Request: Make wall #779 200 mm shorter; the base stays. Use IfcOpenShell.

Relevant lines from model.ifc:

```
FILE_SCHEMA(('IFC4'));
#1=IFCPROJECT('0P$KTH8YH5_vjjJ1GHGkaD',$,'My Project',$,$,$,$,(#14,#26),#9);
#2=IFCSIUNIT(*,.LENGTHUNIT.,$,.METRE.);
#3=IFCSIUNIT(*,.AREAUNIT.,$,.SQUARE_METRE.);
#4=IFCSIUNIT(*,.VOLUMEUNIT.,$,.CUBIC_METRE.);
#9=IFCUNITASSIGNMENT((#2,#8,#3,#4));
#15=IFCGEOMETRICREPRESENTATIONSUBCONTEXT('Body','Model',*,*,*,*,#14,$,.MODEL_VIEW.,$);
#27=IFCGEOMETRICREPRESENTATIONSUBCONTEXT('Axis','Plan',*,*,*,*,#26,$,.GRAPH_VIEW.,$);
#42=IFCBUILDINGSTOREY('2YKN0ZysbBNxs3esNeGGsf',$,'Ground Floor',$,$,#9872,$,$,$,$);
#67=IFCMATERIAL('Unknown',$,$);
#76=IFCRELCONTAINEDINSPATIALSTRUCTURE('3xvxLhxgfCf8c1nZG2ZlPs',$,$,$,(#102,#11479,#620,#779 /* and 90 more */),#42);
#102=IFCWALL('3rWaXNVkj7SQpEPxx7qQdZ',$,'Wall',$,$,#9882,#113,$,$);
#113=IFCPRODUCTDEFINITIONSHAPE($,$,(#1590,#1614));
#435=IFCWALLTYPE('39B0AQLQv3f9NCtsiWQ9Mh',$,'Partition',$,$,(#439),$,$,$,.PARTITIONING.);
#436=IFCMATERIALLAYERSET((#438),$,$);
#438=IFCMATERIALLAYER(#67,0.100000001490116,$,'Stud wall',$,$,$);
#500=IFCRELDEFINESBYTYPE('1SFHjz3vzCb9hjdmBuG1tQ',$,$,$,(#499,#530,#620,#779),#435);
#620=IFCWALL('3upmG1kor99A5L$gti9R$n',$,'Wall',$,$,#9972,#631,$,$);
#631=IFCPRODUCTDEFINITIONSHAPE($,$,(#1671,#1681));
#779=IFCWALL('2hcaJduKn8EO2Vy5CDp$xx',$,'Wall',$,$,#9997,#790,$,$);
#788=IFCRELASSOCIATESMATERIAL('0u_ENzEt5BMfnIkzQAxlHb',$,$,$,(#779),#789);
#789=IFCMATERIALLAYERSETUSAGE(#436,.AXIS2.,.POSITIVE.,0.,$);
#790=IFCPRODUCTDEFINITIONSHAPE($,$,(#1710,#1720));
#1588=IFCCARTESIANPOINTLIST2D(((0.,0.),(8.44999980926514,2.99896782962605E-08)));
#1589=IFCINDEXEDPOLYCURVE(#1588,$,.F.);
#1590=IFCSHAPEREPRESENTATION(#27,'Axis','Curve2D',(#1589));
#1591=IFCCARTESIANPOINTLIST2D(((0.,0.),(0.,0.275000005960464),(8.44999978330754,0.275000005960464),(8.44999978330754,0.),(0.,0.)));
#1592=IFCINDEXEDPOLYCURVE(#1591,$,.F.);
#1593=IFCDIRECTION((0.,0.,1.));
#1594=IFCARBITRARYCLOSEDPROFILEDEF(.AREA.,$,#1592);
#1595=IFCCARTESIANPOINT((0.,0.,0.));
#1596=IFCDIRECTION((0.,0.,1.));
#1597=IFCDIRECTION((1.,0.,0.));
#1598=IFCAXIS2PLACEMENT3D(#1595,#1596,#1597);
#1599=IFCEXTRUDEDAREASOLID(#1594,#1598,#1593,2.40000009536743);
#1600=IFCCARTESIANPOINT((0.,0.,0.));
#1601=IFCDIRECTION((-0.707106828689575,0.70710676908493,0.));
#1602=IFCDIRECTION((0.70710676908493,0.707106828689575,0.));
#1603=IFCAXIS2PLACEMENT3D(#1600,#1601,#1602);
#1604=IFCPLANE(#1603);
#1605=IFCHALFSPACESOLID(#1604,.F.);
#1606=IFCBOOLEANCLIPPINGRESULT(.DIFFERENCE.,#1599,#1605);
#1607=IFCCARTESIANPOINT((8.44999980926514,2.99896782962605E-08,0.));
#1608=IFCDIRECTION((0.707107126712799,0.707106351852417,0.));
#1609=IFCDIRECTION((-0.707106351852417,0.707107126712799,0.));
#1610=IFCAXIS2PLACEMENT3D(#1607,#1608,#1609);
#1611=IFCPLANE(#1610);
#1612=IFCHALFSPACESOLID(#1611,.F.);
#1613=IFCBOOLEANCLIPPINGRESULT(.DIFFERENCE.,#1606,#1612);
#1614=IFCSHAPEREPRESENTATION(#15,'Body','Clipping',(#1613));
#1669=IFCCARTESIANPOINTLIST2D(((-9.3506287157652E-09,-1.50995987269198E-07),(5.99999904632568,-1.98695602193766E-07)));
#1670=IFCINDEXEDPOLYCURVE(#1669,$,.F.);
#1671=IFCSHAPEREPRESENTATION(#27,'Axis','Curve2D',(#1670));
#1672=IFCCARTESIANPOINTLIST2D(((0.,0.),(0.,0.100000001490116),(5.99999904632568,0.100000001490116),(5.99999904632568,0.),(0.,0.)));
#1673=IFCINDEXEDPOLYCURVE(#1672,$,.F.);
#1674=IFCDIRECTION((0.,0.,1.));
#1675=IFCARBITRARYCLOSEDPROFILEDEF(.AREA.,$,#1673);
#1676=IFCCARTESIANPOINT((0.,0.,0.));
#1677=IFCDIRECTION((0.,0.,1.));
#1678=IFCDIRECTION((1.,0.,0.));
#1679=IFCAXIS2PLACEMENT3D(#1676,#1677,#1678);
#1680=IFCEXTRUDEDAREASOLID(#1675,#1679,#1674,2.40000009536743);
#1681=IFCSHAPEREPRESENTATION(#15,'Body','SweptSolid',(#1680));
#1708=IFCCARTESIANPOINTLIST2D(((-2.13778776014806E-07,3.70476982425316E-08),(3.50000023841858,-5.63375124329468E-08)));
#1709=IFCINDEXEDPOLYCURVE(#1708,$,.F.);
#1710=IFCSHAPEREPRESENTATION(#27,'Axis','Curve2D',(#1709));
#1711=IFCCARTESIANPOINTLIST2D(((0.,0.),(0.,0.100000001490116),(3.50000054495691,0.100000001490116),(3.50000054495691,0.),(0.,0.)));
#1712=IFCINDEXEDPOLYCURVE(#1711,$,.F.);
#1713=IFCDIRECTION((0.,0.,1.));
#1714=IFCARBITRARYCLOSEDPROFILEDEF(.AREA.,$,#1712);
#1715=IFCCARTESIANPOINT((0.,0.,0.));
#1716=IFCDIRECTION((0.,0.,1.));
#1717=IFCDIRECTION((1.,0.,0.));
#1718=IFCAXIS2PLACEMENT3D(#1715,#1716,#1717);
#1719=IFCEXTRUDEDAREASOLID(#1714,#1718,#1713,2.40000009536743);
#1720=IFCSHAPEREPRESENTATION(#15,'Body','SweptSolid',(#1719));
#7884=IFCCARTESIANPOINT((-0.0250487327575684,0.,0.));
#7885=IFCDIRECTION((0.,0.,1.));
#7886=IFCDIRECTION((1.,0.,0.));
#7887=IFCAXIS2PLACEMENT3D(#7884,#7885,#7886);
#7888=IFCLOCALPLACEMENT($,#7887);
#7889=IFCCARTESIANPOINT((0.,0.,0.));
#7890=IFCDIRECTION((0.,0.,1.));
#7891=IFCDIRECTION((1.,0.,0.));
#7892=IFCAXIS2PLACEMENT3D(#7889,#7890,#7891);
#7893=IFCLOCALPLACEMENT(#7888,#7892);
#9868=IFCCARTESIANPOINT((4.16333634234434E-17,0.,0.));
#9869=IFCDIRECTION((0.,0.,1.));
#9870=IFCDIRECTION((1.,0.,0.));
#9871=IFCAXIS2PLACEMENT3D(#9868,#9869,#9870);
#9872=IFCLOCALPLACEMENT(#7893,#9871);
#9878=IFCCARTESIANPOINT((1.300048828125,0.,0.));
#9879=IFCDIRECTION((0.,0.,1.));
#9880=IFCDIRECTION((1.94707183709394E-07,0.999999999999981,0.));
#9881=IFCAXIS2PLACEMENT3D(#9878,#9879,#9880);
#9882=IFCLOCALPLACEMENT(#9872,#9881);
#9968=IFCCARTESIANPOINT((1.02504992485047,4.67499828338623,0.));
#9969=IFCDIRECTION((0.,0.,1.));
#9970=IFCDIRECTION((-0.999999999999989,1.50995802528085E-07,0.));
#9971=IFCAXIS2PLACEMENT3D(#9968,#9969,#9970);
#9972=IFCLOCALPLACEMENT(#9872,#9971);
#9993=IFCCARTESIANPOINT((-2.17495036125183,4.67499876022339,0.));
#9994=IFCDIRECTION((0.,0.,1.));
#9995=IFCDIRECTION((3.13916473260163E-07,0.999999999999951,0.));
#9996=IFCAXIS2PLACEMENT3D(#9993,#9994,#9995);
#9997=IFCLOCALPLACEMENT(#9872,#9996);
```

```python
import ifcopenshell
import ifcopenshell.geom
import ifcopenshell.util.representation
import ifcopenshell.util.shape
import ifcopenshell.util.unit

model = ifcopenshell.open("model.ifc")
unit_scale = ifcopenshell.util.unit.calculate_unit_scale(model)
settings = ifcopenshell.geom.settings()


def volume(element):
    """Net volume in cubic metres, openings subtracted."""
    shape = ifcopenshell.geom.create_shape(settings, element)
    return ifcopenshell.util.shape.get_volume(shape.geometry)


wall = model.by_id(779)
before = volume(wall)

body = ifcopenshell.util.representation.get_representation(wall, "Model", "Body")
solid = body.Items[0]
old_height = solid.Depth
solid.Depth -= 0.2 / unit_scale
after = volume(wall)

print(f"height {old_height:g} -> {solid.Depth:g}, volume {before:.3f} -> {after:.3f} m3")

model.write("model_edited.ifc")
```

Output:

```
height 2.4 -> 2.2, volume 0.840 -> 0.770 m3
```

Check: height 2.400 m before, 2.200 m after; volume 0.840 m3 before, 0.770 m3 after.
